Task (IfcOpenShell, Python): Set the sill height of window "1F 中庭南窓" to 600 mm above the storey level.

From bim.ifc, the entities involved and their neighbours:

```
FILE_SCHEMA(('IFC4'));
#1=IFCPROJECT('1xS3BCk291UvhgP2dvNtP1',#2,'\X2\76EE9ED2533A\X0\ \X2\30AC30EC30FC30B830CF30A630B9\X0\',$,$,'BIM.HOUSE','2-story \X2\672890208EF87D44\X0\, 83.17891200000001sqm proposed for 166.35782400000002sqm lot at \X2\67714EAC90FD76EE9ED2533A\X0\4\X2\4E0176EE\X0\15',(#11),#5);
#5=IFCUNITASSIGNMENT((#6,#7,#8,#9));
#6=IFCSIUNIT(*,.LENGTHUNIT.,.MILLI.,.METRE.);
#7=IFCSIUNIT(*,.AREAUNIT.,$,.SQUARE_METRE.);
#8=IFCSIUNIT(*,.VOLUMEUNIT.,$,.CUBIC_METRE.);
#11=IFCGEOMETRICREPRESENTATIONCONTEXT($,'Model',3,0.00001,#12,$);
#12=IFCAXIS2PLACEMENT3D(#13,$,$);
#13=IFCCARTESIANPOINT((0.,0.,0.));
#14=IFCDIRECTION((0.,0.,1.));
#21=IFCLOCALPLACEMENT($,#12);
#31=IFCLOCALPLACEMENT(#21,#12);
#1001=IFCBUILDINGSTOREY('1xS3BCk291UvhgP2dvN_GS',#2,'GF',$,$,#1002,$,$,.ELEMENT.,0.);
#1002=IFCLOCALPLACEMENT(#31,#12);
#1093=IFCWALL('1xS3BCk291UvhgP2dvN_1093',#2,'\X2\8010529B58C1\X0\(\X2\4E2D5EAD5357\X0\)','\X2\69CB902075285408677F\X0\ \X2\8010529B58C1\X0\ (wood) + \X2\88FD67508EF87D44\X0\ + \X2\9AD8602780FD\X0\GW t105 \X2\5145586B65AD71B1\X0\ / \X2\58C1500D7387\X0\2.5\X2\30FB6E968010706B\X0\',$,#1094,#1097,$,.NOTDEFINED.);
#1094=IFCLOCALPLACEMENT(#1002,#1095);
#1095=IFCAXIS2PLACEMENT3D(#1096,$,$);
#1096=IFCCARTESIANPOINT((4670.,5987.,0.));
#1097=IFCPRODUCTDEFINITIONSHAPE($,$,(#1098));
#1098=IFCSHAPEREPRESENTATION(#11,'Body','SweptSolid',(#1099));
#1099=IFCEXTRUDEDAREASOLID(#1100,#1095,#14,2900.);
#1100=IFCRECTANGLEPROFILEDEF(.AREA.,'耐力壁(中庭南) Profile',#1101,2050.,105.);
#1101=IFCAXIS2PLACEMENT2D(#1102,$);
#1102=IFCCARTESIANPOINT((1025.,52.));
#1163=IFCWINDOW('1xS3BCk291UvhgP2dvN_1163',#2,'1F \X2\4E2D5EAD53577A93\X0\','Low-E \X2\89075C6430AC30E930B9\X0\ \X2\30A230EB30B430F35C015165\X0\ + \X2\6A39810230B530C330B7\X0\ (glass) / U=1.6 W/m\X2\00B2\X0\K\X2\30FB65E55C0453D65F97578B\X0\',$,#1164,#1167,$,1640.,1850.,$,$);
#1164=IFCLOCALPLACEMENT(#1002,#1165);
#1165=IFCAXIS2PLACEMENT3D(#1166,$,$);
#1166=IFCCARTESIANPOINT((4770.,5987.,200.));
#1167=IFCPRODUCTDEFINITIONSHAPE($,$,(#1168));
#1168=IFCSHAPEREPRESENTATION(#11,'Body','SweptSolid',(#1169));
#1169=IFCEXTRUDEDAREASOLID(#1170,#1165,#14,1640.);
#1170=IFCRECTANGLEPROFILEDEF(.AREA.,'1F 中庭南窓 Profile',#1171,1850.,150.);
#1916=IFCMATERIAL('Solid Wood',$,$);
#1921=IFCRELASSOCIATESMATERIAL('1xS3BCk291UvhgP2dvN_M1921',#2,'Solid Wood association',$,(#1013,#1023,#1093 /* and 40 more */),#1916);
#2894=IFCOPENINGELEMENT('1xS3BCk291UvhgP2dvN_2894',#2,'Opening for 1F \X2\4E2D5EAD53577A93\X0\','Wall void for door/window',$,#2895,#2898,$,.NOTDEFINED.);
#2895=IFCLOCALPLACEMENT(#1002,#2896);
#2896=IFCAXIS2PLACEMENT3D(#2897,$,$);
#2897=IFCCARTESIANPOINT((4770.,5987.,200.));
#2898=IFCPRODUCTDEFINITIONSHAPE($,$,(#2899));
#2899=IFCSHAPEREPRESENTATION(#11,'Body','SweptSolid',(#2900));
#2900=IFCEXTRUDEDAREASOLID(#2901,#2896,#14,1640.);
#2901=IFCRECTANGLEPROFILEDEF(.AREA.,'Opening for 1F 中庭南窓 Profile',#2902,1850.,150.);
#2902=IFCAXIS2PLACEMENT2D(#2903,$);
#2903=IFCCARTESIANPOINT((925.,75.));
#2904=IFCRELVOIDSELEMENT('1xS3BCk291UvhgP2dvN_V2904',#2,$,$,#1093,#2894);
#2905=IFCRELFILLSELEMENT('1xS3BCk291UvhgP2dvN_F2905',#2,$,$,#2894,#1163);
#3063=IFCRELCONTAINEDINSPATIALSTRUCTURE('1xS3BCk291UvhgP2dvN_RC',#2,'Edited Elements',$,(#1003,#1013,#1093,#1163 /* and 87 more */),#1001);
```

```python
import numpy as np
import ifcopenshell
import ifcopenshell.api.geometry
import ifcopenshell.geom
import ifcopenshell.util.element
import ifcopenshell.util.placement
import ifcopenshell.util.shape
import ifcopenshell.util.unit

model = ifcopenshell.open("bim.ifc")
unit_scale = ifcopenshell.util.unit.calculate_unit_scale(model)

window = model.by_id(1163)
opening = window.FillsVoids[0].RelatingOpeningElement
storey = ifcopenshell.util.element.get_container(window, ifc_class="IfcBuildingStorey")
level = ifcopenshell.util.placement.get_local_placement(storey.ObjectPlacement)[2, 3]

# The opening's origin need not be at the sill, so measure its lowest point.
shape = ifcopenshell.geom.create_shape(ifcopenshell.geom.settings(), opening)
bottom = ifcopenshell.util.shape.get_shape_bottom_elevation(shape, shape.geometry) / unit_scale
dz = level + 0.6 / unit_scale - bottom

shift = np.array([0.0, 0.0, dz])
# The window is not placed relative to its opening, so move both.
for product in (opening, window):
    matrix = ifcopenshell.util.placement.get_local_placement(product.ObjectPlacement)
    matrix[:3, 3] += shift
    ifcopenshell.api.geometry.edit_object_placement(model, product=product, matrix=matrix, is_si=False)

print(f"moved by {dz * unit_scale:+.3f} m")

model.write("bim_rev.ifc")
```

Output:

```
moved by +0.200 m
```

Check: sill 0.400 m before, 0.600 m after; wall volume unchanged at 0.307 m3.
